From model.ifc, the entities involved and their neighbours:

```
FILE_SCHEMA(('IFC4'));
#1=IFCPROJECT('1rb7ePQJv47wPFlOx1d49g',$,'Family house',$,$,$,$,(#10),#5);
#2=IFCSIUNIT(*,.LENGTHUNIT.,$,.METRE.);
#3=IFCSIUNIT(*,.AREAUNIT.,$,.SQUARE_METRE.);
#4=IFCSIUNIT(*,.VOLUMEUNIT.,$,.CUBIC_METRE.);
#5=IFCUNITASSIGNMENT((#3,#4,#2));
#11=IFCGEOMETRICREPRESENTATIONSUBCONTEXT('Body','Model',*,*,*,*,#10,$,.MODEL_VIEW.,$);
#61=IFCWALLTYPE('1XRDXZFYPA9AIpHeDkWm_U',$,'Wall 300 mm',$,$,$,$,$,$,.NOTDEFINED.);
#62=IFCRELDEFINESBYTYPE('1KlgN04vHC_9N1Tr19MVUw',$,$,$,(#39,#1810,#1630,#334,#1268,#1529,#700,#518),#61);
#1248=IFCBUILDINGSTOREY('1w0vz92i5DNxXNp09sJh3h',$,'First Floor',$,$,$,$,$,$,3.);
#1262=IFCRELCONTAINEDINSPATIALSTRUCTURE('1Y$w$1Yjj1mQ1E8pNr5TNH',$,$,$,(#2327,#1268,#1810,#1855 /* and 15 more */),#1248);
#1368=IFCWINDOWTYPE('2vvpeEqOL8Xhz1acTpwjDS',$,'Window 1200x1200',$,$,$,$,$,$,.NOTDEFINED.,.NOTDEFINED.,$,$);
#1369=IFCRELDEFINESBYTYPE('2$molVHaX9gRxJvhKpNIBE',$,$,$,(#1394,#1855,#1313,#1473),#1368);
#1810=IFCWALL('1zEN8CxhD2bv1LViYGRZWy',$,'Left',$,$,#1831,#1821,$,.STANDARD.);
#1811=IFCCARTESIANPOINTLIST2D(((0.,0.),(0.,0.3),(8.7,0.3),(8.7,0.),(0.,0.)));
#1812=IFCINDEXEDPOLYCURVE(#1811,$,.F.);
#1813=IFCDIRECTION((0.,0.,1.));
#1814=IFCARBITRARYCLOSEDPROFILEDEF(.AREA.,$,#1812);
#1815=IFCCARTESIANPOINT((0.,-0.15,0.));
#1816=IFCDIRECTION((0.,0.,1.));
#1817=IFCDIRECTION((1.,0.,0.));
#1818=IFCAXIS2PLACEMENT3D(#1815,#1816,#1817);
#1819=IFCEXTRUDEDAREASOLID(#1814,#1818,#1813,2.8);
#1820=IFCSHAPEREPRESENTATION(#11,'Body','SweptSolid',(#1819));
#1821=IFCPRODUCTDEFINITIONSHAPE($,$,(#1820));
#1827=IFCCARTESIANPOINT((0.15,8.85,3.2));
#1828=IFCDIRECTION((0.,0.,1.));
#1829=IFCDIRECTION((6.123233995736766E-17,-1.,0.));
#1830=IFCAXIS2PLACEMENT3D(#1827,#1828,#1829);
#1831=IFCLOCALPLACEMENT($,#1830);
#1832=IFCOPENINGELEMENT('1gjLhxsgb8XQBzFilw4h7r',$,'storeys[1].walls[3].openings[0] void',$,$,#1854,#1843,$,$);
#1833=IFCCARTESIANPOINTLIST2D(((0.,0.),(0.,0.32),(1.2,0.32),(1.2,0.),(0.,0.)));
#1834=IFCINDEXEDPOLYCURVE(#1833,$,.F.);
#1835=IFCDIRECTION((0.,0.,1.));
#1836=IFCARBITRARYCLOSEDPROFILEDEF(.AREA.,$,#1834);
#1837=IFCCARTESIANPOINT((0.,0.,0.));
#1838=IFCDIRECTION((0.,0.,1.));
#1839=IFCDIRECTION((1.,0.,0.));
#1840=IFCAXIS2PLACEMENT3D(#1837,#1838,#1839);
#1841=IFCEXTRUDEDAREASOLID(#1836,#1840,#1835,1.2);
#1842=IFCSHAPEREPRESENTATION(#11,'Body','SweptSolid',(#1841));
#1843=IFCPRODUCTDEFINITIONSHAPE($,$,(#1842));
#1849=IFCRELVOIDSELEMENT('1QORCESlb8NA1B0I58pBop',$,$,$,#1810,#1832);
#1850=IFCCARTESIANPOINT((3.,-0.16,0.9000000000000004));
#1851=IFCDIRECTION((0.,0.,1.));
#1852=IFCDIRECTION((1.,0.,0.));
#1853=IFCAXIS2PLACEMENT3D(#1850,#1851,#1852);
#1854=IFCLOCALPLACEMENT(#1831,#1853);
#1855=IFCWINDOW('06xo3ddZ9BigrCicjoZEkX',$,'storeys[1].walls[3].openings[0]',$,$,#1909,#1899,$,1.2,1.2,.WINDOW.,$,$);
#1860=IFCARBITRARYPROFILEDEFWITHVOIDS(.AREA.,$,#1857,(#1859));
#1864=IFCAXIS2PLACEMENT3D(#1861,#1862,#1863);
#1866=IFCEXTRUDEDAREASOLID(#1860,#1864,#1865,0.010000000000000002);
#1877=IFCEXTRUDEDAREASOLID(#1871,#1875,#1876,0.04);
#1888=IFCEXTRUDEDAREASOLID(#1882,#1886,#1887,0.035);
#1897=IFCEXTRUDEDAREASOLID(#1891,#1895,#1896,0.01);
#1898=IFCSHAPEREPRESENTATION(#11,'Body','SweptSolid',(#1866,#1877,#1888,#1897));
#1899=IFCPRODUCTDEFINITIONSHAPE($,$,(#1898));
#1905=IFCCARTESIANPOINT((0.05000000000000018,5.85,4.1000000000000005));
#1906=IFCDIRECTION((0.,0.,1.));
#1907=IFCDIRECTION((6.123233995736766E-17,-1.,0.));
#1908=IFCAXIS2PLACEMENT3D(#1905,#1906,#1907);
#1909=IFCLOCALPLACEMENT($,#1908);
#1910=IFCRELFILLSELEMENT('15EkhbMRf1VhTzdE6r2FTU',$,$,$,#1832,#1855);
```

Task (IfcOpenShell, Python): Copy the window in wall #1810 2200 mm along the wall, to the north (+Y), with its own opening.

```python
import ifcopenshell
import ifcopenshell.api.feature
import ifcopenshell.api.geometry
import ifcopenshell.api.root
import ifcopenshell.geom
import ifcopenshell.util.element
import ifcopenshell.util.placement
import ifcopenshell.util.shape
import ifcopenshell.util.unit

model = ifcopenshell.open("model.ifc")
unit_scale = ifcopenshell.util.unit.calculate_unit_scale(model)
settings = ifcopenshell.geom.settings()


def volume(element):
    """Net volume in cubic metres, openings subtracted."""
    shape = ifcopenshell.geom.create_shape(settings, element)
    return ifcopenshell.util.shape.get_volume(shape.geometry)


window = model.by_guid("06xo3ddZ9BigrCicjoZEkX")
opening = window.FillsVoids[0].RelatingOpeningElement
wall = opening.VoidsElements[0].RelatingBuildingElement
before = volume(wall)
shift = ifcopenshell.util.placement.get_local_placement(wall.ObjectPlacement)[:3, 0] * -2.2 / unit_scale

# copy_class copies the void relationship, type, container and properties, but no geometry.
new_opening = ifcopenshell.api.root.copy_class(model, product=opening)
new_opening.Representation = ifcopenshell.util.element.copy_deep(
    model, opening.Representation, exclude=["IfcGeometricRepresentationContext", "IfcRepresentationMap"]
)
new_window = ifcopenshell.api.root.copy_class(model, product=window)
new_window.Representation = ifcopenshell.util.element.copy_deep(
    model, window.Representation, exclude=["IfcGeometricRepresentationContext", "IfcRepresentationMap"]
)
ifcopenshell.api.feature.add_filling(model, opening=new_opening, element=new_window)

for old, new in ((opening, new_opening), (window, new_window)):
    matrix = ifcopenshell.util.placement.get_local_placement(old.ObjectPlacement)
    matrix[:3, 3] += shift
    ifcopenshell.api.geometry.edit_object_placement(model, product=new, matrix=matrix, is_si=False)

after = volume(wall)

print(f"wall volume {before:.3f} -> {after:.3f} m3")

model.write("model-out.ifc")
```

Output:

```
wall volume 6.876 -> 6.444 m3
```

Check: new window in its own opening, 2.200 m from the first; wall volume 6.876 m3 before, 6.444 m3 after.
